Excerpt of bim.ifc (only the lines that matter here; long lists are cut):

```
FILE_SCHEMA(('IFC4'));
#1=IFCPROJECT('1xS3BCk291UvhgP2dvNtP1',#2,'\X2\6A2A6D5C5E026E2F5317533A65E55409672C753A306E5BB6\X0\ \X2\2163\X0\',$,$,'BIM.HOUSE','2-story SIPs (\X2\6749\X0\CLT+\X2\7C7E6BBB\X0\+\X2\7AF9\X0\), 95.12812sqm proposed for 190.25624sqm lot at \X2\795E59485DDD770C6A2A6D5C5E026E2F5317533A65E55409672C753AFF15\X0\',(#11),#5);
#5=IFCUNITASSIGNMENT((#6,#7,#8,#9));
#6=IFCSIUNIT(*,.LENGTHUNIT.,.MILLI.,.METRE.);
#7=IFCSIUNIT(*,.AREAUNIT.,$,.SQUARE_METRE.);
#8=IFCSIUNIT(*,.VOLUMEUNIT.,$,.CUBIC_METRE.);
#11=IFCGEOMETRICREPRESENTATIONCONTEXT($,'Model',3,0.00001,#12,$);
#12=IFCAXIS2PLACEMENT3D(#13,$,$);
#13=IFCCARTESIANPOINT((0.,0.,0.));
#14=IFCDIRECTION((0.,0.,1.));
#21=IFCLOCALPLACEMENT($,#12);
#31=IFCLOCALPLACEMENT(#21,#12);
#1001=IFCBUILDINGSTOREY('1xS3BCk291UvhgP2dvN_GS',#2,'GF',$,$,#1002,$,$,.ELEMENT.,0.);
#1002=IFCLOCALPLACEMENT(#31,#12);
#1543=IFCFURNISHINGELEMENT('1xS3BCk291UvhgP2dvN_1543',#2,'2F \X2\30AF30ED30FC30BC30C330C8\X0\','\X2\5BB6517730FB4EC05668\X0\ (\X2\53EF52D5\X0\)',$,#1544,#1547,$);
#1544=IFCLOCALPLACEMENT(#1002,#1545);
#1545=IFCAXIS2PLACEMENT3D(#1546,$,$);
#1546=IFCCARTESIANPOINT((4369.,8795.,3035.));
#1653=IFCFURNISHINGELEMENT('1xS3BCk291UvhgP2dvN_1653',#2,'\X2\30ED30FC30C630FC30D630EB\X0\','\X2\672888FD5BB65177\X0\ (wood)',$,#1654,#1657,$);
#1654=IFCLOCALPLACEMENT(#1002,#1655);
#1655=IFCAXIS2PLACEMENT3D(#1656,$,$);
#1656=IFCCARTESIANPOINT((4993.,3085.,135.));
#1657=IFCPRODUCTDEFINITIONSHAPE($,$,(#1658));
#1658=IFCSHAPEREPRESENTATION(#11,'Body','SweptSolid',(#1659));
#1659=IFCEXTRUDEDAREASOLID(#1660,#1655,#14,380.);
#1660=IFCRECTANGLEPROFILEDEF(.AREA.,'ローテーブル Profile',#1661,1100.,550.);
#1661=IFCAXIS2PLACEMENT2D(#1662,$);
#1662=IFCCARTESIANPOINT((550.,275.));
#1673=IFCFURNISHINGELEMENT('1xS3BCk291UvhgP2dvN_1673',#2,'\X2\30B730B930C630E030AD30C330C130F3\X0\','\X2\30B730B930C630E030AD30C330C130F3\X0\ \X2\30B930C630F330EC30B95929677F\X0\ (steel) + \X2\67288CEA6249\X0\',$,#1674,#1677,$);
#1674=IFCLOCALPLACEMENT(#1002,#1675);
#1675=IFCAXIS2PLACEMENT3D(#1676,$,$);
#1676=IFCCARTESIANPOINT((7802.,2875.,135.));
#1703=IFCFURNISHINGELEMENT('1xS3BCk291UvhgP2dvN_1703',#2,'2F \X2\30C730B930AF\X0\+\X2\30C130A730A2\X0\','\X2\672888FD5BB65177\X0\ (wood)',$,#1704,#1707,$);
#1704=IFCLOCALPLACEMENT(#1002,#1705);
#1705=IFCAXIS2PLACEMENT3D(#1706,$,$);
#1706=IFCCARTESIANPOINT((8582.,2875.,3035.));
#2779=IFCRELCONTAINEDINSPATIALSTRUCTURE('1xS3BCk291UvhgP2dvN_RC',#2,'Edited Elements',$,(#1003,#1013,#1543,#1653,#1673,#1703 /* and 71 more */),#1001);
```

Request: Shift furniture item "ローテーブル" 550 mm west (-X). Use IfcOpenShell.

```python
import ifcopenshell
import ifcopenshell.api.geometry
import ifcopenshell.util.placement

model = ifcopenshell.open("bim.ifc")

item = model.by_guid("1xS3BCk291UvhgP2dvN_1653")
matrix = ifcopenshell.util.placement.get_local_placement(item.ObjectPlacement)
matrix[0, 3] -= 550.0
ifcopenshell.api.geometry.edit_object_placement(model, product=item, matrix=matrix, is_si=False)

print(ifcopenshell.util.placement.get_local_placement(item.ObjectPlacement).round(3) + 0.0)

model.write("bim_rev.ifc")
```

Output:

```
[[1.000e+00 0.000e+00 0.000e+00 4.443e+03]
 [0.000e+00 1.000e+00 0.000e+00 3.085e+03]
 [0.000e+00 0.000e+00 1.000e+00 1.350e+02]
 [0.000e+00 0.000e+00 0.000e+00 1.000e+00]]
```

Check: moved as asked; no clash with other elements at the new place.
